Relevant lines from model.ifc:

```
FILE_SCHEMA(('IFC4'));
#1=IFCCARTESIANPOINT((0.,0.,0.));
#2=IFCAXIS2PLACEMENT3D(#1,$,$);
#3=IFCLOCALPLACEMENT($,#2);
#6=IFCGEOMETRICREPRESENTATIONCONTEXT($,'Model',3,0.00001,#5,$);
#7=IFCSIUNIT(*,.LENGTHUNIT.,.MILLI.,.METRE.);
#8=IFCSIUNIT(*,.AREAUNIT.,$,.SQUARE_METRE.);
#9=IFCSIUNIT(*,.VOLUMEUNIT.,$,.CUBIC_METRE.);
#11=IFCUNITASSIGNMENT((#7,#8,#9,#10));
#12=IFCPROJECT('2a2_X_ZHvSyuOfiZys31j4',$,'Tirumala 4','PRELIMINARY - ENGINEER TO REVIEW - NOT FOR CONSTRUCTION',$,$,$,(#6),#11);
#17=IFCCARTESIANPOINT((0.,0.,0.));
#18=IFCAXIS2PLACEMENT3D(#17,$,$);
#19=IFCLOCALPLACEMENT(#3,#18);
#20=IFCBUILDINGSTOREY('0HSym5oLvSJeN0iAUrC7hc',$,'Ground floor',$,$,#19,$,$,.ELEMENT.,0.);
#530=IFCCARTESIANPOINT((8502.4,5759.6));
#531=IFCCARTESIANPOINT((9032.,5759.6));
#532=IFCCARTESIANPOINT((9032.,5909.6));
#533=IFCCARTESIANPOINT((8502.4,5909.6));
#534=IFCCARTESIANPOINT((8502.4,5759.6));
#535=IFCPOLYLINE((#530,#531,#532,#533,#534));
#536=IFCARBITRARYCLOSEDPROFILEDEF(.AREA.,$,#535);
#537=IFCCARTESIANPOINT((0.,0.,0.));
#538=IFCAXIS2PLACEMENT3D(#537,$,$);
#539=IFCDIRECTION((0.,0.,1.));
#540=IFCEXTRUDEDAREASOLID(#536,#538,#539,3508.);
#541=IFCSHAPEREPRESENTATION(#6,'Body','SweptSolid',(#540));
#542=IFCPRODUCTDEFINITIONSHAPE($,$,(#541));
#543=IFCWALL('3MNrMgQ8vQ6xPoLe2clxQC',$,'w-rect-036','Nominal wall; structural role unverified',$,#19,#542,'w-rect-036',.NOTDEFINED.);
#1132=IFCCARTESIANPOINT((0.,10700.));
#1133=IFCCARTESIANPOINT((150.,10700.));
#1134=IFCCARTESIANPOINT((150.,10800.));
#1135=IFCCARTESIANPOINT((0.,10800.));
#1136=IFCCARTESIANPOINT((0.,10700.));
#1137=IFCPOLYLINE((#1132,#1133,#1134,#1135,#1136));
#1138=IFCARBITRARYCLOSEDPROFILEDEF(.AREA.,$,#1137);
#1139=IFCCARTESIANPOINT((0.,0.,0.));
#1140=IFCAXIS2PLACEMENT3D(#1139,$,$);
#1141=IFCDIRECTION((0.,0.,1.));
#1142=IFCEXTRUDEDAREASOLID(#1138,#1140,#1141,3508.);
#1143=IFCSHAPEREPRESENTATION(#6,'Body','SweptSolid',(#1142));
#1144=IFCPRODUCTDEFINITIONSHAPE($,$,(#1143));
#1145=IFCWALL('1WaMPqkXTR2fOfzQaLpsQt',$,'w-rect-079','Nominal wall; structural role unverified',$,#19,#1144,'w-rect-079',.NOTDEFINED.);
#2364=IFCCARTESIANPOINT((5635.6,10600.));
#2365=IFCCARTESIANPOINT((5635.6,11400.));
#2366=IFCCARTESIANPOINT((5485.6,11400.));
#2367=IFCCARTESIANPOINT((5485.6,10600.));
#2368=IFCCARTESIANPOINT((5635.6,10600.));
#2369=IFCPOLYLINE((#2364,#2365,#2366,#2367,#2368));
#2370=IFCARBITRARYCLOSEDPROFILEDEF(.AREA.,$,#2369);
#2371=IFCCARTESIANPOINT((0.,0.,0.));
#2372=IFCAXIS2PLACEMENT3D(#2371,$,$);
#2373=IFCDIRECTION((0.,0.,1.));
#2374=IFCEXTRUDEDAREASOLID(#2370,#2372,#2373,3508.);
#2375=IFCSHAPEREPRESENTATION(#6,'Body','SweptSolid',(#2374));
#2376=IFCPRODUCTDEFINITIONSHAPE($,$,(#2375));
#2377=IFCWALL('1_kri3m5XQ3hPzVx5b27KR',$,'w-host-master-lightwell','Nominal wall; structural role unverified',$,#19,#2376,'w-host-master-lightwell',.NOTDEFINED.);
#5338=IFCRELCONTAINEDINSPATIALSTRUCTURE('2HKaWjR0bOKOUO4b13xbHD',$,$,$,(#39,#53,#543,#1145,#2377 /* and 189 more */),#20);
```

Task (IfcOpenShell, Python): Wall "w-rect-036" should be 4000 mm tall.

```python
import ifcopenshell
import ifcopenshell.geom
import ifcopenshell.util.shape
import ifcopenshell.util.unit

model = ifcopenshell.open("model.ifc")
unit_scale = ifcopenshell.util.unit.calculate_unit_scale(model)
settings = ifcopenshell.geom.settings()


def volume(element):
    """Net volume in cubic metres, openings subtracted."""
    shape = ifcopenshell.geom.create_shape(settings, element)
    return ifcopenshell.util.shape.get_volume(shape.geometry)


wall = model.by_guid("3MNrMgQ8vQ6xPoLe2clxQC")
before = volume(wall)

body = next(r for r in wall.Representation.Representations if r.RepresentationIdentifier == "Body")
solid = body.Items[0]
old_height = solid.Depth
solid.Depth = 4 / unit_scale
after = volume(wall)

print(f"height {old_height:g} -> {solid.Depth:g}, volume {before:.3f} -> {after:.3f} m3")

model.write("model_edited.ifc")
```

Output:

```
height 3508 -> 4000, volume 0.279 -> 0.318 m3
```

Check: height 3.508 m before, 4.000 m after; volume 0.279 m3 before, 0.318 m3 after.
